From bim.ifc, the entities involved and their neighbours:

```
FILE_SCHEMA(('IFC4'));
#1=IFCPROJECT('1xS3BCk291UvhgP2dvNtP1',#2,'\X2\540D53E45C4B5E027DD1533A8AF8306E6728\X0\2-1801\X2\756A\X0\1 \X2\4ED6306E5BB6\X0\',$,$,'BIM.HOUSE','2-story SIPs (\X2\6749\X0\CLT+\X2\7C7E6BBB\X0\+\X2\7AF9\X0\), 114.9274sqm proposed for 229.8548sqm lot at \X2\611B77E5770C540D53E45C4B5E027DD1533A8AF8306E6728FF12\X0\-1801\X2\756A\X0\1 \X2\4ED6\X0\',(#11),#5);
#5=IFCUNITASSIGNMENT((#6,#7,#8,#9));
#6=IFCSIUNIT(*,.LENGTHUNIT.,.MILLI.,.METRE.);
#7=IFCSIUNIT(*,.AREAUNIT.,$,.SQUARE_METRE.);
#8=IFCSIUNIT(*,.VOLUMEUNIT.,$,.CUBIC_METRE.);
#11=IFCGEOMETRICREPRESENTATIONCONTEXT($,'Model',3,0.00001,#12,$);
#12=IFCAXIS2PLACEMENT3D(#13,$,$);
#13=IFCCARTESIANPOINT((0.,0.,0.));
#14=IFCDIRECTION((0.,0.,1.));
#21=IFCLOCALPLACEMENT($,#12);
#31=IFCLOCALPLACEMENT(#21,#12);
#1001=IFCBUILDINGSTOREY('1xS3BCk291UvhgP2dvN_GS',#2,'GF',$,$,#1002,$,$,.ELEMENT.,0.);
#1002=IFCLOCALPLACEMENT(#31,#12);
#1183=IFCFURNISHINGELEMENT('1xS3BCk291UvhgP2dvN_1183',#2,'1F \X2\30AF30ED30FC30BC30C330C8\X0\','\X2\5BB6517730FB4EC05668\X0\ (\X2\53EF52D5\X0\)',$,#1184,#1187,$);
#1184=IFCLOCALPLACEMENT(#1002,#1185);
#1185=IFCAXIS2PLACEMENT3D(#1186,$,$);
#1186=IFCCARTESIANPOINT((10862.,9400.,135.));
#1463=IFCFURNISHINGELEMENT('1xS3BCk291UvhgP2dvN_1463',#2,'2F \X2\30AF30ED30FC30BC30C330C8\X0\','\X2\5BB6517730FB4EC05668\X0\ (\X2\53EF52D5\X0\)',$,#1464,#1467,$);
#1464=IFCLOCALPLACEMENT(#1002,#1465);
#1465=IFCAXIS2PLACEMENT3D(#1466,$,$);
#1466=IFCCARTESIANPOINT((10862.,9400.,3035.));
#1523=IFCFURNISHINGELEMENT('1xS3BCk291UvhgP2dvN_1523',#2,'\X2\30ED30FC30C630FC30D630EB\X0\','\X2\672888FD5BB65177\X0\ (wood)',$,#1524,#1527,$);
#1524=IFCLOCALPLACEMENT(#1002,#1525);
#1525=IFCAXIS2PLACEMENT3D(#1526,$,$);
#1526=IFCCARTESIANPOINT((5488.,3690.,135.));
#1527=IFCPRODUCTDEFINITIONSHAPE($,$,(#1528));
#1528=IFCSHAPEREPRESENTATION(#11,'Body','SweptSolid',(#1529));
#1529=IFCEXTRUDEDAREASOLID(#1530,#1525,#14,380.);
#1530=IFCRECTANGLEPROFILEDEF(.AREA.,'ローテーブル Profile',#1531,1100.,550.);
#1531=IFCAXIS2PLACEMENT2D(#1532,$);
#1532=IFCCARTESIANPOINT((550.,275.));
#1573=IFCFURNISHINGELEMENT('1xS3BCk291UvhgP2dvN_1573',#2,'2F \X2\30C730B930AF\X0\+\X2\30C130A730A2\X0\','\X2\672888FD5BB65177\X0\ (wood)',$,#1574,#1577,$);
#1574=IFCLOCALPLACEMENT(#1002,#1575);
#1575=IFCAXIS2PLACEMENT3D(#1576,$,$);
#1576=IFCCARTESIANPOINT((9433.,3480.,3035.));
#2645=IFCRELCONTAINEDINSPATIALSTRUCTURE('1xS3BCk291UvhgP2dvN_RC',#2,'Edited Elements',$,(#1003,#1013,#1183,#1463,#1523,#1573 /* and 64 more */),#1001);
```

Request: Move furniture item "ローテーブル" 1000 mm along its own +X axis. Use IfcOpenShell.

```python
import ifcopenshell
import ifcopenshell.api.geometry
import ifcopenshell.util.placement
import ifcopenshell.util.unit

model = ifcopenshell.open("bim.ifc")
unit_scale = ifcopenshell.util.unit.calculate_unit_scale(model)

item = model.by_guid("1xS3BCk291UvhgP2dvN_1523")
matrix = ifcopenshell.util.placement.get_local_placement(item.ObjectPlacement)
matrix[:3, 3] += matrix[:3, 0] * 1 / unit_scale
ifcopenshell.api.geometry.edit_object_placement(model, product=item, matrix=matrix, is_si=False)

print(ifcopenshell.util.placement.get_local_placement(item.ObjectPlacement).round(3) + 0.0)

model.write("bim-out.ifc")
```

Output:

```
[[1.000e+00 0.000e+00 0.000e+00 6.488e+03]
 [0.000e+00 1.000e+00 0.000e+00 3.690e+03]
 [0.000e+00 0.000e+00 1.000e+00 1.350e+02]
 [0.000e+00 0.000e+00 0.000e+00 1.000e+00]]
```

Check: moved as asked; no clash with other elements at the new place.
